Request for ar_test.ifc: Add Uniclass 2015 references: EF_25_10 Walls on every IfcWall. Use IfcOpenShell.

First a look at what the model holds.

```python
import ifcopenshell

model = ifcopenshell.open("ar_test.ifc")
print(model.schema)
print("classifications:", [c.Name for c in model.by_type("IfcClassification")])
for ifc_class in ("IfcDoor", "IfcRoof", "IfcStair", "IfcWall", "IfcWindow"):
    print(ifc_class, len(model.by_type(ifc_class)))
```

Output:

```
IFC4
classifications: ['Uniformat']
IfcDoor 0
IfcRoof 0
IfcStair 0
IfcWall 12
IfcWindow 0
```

```python
import ifcopenshell
import ifcopenshell.api.classification

model = ifcopenshell.open("ar_test.ifc")

system = ifcopenshell.api.classification.add_classification(model, classification="Uniclass 2015")

codes = {
    "IfcWall": ("EF_25_10", "Walls"),
}
for ifc_class, (code, name) in codes.items():
    products = model.by_type(ifc_class)
    ifcopenshell.api.classification.add_reference(
        model, products=products, classification=system, identification=code, name=name
    )
    print(code, len(products))

model.write("ar_test-out.ifc")
```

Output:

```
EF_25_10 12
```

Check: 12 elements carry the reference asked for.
